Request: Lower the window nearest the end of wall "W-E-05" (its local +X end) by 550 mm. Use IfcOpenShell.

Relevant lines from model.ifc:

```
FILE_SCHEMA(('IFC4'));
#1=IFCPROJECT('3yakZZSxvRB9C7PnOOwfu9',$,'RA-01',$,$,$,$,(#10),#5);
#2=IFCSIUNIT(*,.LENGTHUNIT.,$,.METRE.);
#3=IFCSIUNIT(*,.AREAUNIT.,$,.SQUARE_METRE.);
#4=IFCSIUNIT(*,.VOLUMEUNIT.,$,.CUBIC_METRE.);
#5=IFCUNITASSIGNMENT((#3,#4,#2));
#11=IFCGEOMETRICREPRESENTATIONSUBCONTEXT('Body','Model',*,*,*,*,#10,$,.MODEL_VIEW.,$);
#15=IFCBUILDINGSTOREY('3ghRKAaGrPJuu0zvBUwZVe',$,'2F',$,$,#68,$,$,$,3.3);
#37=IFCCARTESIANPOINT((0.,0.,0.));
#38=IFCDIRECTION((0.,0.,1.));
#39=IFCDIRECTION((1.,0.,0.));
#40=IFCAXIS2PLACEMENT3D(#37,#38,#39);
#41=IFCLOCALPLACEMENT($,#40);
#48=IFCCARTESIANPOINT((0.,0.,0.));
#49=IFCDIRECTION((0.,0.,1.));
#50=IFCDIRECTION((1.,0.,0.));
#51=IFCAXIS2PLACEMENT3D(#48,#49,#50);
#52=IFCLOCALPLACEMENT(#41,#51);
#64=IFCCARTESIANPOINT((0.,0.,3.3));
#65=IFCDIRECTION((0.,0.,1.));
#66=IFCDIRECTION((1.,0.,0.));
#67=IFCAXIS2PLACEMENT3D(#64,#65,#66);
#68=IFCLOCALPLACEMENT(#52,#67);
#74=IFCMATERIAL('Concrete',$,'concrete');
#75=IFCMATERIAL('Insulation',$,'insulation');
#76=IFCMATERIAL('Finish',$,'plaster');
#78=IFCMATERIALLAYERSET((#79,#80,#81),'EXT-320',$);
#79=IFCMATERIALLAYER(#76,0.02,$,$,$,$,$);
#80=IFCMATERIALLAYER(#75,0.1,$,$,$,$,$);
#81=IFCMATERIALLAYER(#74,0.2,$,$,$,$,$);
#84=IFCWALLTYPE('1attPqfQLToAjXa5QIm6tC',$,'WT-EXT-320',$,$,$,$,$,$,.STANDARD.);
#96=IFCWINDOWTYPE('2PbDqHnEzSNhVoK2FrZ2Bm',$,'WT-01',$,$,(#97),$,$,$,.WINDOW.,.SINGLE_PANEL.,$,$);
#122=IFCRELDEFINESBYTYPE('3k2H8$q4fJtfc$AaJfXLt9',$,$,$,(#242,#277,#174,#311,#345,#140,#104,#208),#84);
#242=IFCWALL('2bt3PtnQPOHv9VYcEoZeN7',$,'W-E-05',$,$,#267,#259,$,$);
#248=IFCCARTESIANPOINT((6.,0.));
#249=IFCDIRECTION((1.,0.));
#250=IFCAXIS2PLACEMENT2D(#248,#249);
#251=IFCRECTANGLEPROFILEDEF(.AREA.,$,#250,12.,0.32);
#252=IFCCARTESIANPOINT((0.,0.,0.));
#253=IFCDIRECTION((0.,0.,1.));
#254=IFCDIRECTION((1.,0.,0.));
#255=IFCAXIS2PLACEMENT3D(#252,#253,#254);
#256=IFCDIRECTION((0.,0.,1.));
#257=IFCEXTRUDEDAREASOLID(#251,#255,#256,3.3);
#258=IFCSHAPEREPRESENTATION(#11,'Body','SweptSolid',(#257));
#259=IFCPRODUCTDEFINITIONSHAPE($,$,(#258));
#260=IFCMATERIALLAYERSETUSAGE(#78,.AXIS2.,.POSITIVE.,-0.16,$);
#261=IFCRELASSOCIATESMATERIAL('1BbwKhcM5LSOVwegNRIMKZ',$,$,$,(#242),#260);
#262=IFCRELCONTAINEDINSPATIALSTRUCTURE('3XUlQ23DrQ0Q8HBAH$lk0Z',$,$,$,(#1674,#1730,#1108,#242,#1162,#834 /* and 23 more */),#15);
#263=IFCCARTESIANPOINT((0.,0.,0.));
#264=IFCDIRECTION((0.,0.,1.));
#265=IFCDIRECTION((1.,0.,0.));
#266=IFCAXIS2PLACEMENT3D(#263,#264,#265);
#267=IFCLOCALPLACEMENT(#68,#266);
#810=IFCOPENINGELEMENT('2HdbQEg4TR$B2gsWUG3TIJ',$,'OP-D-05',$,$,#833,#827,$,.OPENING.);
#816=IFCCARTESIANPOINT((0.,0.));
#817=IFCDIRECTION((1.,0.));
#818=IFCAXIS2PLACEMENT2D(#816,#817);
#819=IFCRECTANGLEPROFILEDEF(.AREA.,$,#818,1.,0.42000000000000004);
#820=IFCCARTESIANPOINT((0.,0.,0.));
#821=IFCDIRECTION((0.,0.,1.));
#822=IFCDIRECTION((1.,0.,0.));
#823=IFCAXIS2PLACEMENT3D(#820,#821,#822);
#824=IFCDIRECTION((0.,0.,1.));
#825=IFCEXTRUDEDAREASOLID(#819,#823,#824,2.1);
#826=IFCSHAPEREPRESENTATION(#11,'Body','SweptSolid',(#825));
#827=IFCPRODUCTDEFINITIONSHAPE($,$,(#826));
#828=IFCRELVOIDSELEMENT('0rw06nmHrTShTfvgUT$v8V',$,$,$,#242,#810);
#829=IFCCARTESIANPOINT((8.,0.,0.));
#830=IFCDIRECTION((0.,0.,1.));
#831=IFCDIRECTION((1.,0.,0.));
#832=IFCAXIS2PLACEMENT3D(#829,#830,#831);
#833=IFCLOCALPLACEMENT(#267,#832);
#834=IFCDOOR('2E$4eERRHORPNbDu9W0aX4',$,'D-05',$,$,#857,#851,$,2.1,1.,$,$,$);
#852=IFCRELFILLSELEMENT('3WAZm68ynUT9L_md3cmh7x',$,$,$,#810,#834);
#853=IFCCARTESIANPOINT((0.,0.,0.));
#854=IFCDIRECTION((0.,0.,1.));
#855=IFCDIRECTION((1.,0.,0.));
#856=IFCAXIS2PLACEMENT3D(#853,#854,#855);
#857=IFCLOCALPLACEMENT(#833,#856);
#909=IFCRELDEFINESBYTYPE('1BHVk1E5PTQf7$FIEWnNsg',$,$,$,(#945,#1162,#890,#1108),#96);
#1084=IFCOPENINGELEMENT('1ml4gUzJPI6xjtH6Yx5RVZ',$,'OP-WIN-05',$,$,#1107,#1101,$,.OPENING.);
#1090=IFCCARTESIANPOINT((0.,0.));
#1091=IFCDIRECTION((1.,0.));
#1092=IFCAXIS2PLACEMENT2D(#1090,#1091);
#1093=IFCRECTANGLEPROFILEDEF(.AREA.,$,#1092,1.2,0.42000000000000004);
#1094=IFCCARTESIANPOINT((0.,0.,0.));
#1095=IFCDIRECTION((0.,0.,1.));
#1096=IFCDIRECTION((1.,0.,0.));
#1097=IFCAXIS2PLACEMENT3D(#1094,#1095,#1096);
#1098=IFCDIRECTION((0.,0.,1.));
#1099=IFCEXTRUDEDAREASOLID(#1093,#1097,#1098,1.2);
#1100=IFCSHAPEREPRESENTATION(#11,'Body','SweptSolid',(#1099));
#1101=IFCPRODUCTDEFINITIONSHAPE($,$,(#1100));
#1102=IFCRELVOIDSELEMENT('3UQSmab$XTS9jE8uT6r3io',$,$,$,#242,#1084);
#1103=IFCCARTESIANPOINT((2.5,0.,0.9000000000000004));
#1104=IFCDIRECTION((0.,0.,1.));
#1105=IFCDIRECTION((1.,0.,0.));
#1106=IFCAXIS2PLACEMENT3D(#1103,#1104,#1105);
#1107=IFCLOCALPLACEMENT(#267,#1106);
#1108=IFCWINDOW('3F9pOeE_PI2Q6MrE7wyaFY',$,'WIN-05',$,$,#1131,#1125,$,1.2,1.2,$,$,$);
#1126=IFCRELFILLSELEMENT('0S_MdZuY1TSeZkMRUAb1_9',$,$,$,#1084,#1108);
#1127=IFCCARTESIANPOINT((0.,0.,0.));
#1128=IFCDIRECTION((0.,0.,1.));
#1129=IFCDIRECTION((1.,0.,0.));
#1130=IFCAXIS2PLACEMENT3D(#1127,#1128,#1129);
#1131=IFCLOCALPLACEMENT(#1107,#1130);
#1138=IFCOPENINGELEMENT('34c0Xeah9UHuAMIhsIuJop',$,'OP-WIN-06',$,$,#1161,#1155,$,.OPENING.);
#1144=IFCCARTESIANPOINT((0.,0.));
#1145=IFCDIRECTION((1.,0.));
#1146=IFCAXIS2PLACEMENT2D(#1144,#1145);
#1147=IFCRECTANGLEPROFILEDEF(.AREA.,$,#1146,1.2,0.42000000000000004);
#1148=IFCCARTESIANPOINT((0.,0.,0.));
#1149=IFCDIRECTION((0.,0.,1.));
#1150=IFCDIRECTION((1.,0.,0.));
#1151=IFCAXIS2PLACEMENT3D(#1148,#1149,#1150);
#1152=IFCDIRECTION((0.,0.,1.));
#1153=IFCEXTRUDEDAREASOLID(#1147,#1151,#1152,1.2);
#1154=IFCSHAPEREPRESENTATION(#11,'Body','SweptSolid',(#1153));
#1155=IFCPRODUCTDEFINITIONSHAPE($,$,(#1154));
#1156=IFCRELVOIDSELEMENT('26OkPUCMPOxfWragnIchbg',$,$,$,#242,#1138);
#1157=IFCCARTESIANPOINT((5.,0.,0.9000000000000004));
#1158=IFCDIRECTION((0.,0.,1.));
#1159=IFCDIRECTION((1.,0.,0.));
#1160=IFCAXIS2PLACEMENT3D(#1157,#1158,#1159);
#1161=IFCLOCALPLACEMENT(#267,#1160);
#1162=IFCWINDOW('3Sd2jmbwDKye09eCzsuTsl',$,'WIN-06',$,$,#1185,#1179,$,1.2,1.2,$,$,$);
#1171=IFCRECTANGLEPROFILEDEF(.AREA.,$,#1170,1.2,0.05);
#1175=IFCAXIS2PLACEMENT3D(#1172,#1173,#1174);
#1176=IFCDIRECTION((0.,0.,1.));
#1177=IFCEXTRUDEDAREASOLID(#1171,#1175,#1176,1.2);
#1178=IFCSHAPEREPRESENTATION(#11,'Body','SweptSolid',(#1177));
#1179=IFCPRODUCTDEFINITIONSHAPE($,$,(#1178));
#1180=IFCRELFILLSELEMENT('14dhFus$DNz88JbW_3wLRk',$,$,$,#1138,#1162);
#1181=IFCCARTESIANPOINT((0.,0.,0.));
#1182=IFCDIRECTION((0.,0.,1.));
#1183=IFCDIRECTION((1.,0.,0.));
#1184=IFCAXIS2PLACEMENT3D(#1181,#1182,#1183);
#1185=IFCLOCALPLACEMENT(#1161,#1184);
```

```python
import numpy as np
import ifcopenshell
import ifcopenshell.api.geometry
import ifcopenshell.util.placement
import ifcopenshell.util.unit

model = ifcopenshell.open("model.ifc")
unit_scale = ifcopenshell.util.unit.calculate_unit_scale(model)

window = model.by_guid("3Sd2jmbwDKye09eCzsuTsl")
opening = window.FillsVoids[0].RelatingOpeningElement
dz = -0.55 / unit_scale

shift = np.array([0.0, 0.0, dz])
# The window is placed relative to its opening, so it follows when the opening moves.
matrix = ifcopenshell.util.placement.get_local_placement(opening.ObjectPlacement)
matrix[:3, 3] += shift
ifcopenshell.api.geometry.edit_object_placement(
    model, product=opening, matrix=matrix, is_si=False, should_transform_children=True
)

print(f"moved by {dz * unit_scale:+.3f} m")

model.write("model_updated.ifc")
```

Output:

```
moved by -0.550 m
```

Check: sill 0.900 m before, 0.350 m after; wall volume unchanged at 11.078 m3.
